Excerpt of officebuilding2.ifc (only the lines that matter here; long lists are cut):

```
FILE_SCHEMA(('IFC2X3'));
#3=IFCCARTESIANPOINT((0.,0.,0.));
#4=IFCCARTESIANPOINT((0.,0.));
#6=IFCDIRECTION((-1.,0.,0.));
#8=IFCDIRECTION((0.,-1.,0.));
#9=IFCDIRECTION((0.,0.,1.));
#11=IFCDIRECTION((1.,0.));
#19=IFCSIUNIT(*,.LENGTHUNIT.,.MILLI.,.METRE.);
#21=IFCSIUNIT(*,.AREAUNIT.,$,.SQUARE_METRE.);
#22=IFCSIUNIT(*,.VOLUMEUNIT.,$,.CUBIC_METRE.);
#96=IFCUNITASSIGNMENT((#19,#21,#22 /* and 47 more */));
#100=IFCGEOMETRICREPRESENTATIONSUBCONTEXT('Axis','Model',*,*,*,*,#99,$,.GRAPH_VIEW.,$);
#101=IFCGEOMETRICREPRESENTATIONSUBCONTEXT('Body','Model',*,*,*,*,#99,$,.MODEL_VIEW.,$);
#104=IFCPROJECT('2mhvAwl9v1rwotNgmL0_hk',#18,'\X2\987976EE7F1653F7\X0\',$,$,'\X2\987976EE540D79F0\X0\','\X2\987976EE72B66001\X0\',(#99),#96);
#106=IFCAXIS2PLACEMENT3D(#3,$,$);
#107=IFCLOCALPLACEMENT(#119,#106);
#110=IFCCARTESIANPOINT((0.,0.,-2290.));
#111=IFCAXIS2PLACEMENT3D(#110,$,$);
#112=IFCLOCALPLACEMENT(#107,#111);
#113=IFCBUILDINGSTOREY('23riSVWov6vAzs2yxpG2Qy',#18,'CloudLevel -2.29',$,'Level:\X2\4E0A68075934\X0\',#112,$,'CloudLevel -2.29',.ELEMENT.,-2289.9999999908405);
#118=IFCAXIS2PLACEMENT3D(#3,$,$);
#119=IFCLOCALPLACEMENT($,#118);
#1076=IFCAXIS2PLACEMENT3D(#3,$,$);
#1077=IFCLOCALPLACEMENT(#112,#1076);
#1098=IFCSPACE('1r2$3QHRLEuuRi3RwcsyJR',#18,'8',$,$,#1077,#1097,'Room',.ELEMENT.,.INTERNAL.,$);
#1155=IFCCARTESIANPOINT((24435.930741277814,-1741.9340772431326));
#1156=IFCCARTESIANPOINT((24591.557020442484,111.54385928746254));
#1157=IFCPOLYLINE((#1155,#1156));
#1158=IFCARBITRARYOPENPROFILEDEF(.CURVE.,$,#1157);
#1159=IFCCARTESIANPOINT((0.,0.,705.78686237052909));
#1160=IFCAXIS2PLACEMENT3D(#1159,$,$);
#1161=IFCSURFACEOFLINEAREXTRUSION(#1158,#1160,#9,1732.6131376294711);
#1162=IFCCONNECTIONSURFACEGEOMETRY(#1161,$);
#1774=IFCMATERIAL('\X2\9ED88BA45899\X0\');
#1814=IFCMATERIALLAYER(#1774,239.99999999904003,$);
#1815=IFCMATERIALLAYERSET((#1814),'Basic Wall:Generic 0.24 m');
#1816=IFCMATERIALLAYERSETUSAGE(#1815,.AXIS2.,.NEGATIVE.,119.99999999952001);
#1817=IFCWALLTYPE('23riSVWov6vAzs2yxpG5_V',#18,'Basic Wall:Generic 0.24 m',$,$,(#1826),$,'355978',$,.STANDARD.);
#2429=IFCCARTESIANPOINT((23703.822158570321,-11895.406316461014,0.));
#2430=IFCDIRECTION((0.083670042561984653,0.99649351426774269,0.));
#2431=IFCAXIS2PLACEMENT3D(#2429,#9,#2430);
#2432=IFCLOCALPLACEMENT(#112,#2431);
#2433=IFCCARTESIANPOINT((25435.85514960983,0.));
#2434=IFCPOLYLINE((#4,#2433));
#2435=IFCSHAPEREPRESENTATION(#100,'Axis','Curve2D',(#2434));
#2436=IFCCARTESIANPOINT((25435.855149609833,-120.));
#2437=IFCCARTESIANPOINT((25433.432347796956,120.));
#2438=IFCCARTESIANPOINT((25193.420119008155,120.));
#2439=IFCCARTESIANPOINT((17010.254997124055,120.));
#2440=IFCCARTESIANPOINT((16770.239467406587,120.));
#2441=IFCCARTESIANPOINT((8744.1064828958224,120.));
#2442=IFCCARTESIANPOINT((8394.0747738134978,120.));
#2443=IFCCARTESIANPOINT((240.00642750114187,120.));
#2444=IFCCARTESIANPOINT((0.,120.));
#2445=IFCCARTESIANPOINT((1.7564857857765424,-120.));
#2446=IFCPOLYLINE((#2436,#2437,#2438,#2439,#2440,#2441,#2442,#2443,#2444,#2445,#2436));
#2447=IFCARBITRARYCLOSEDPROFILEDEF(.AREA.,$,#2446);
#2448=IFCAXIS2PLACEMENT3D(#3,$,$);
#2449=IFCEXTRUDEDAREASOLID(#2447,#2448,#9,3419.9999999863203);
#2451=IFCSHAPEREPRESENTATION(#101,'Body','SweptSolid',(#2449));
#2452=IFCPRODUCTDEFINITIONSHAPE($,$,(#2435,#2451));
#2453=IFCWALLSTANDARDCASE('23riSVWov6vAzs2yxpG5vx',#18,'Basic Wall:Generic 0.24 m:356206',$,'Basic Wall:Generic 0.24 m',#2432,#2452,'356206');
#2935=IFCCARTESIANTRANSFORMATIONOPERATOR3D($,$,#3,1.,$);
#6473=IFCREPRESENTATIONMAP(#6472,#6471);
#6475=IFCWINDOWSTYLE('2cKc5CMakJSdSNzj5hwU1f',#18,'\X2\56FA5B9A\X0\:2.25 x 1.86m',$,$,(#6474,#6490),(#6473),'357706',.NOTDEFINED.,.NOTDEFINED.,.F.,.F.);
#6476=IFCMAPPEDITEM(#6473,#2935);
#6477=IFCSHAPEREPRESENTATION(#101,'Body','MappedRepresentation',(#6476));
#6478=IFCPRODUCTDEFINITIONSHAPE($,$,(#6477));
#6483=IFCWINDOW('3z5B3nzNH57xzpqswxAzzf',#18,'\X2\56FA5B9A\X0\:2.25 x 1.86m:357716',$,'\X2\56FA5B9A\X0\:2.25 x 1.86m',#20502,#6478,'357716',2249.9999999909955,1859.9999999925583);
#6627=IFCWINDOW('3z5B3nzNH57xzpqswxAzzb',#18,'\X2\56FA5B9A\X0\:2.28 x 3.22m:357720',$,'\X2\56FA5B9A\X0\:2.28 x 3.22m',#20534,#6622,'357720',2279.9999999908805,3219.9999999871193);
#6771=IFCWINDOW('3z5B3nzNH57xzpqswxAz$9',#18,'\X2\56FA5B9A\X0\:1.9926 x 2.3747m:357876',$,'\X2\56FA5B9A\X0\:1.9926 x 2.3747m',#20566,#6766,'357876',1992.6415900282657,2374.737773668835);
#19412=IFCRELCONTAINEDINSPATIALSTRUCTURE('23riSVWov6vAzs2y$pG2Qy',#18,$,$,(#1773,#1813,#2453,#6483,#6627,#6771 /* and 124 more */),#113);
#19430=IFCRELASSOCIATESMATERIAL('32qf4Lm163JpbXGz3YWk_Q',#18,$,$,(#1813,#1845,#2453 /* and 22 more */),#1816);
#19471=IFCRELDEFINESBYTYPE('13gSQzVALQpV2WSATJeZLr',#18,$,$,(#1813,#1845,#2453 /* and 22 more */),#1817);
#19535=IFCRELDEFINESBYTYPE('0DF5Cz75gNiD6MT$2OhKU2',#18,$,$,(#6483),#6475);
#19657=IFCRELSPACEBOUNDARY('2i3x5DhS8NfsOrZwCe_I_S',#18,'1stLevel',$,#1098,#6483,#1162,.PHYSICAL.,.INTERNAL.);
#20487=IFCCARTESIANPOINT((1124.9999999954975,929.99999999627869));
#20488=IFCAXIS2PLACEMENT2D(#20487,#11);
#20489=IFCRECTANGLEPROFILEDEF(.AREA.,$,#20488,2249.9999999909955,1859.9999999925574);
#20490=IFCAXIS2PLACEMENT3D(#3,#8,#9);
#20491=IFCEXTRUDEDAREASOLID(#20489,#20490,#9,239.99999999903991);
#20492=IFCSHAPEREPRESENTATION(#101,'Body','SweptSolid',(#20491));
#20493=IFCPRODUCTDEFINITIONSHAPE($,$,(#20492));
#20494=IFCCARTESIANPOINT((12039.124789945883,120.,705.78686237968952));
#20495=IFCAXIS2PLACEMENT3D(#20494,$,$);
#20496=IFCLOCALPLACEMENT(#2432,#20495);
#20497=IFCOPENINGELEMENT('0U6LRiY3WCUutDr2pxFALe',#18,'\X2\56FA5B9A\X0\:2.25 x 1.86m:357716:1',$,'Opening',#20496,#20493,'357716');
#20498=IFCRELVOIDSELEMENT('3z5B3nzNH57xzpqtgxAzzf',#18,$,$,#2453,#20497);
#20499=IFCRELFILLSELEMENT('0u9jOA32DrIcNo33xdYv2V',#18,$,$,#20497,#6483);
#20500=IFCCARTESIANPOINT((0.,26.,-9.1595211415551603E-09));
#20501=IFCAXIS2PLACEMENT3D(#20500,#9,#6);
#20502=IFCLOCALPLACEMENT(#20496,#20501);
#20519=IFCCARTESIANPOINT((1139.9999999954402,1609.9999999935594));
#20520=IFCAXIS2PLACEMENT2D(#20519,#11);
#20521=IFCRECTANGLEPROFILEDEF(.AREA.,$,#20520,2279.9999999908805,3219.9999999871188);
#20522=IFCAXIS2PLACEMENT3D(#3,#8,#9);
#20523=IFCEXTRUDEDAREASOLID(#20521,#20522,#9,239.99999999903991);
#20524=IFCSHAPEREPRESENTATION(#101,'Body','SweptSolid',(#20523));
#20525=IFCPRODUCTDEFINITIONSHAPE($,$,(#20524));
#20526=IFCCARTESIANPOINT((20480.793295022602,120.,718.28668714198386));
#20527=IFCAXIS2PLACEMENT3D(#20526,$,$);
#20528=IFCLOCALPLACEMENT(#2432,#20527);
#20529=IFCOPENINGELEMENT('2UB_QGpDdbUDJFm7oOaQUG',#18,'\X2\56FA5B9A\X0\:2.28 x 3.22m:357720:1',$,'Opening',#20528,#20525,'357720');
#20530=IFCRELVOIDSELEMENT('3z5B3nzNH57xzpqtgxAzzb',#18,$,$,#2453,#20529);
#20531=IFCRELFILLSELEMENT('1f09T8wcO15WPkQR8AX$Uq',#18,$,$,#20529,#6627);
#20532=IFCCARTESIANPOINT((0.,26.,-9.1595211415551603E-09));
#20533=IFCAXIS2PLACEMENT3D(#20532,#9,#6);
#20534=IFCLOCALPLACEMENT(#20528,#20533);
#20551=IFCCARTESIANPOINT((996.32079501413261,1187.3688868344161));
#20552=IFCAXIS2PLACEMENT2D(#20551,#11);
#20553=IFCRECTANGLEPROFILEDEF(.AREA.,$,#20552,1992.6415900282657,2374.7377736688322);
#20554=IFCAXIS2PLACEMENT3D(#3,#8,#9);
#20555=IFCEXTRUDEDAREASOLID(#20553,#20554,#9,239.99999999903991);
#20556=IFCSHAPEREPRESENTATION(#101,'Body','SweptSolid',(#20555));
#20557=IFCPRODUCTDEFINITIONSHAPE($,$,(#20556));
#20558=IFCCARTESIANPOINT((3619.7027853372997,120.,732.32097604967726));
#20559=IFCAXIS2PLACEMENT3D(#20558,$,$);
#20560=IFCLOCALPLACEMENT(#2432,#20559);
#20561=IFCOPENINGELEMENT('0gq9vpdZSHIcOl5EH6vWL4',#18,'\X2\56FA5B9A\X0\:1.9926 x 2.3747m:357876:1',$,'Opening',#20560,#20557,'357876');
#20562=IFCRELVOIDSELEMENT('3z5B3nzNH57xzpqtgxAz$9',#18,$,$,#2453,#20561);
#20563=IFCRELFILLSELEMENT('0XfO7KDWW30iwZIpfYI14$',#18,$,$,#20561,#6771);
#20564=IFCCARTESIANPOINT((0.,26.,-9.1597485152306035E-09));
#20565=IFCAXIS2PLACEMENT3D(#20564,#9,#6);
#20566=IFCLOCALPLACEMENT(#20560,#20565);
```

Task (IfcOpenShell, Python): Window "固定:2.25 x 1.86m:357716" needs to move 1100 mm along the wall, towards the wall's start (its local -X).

```python
import numpy as np
import ifcopenshell
import ifcopenshell.api.geometry
import ifcopenshell.util.placement
import ifcopenshell.util.unit

model = ifcopenshell.open("officebuilding2.ifc")
unit_scale = ifcopenshell.util.unit.calculate_unit_scale(model)

window = model.by_guid("3z5B3nzNH57xzpqswxAzzf")
opening = window.FillsVoids[0].RelatingOpeningElement
wall = opening.VoidsElements[0].RelatingBuildingElement

wall_matrix = ifcopenshell.util.placement.get_local_placement(wall.ObjectPlacement)
shift = wall_matrix[:3, 0] * -1.1 / unit_scale
before = ifcopenshell.util.placement.get_local_placement(window.ObjectPlacement)[:3, 3].copy()

# The window is placed relative to its opening, so it follows when the opening moves.
matrix = ifcopenshell.util.placement.get_local_placement(opening.ObjectPlacement)
matrix[:3, 3] += shift
ifcopenshell.api.geometry.edit_object_placement(
    model, product=opening, matrix=matrix, is_si=False, should_transform_children=True
)

# Space boundary surfaces are stored in each space's coordinates; move them too.
for rel in window.ProvidesBoundaries:
    if not rel.ConnectionGeometry:
        continue
    surface = rel.ConnectionGeometry.SurfaceOnRelatingElement
    space_matrix = ifcopenshell.util.placement.get_local_placement(rel.RelatingSpace.ObjectPlacement)
    point = np.array(surface.Position.Location.Coordinates) + space_matrix[:3, :3].T @ shift
    surface.Position = model.createIfcAxis2Placement3D(
        model.createIfcCartesianPoint(point.tolist()), surface.Position.Axis, surface.Position.RefDirection
    )

after = ifcopenshell.util.placement.get_local_placement(window.ObjectPlacement)[:3, 3]
print("window moved by", (after - before).round(3) + 0.0)

model.write("officebuilding2-out.ifc")
```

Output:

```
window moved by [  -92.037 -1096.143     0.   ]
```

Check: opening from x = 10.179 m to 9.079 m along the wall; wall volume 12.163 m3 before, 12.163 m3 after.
